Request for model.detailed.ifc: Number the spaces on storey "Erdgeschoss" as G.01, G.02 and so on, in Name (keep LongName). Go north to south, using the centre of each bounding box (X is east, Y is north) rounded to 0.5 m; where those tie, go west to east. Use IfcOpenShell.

First a look at what the model holds.

```python
import ifcopenshell
import ifcopenshell.util.element
import ifcopenshell.util.placement

model = ifcopenshell.open("model.detailed.ifc")
print(model.schema)
storey = next(s for s in model.by_type("IfcBuildingStorey") if s.Name == "Erdgeschoss")
spaces = [e for e in ifcopenshell.util.element.get_decomposition(storey) if e.is_a("IfcSpace")]
for e in sorted(spaces, key=lambda e: e.id()):
    origin = ifcopenshell.util.placement.get_local_placement(e.ObjectPlacement)[:3, 3]
    print(e.id(), e.Name, e.LongName, origin.round(2) + 0.0, sep=" | ")
```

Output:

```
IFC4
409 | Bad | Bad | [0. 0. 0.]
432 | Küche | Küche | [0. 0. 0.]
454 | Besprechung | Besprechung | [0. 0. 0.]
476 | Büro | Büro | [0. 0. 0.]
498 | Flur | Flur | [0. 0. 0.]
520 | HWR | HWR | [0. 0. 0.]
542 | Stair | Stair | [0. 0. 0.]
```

```python
import ifcopenshell
import ifcopenshell.geom
import ifcopenshell.util.element
import ifcopenshell.util.shape

model = ifcopenshell.open("model.detailed.ifc")
settings = ifcopenshell.geom.settings()
settings.set("use-world-coords", True)


def centre(element):
    shape = ifcopenshell.geom.create_shape(settings, element)
    return ifcopenshell.util.shape.get_bbox_centroid(shape.geometry)


storey = next(s for s in model.by_type("IfcBuildingStorey") if s.Name == "Erdgeschoss")
spaces = [e for e in ifcopenshell.util.element.get_decomposition(storey) if e.is_a("IfcSpace")]

# Insertion points can sit at a corner or the storey origin, so sort by the geometry (in metres).
centres = {e: centre(e) for e in spaces}
spaces.sort(key=lambda e: (-round(centres[e][1] / 0.5), centres[e][0]))

for i, e in enumerate(spaces, start=1):
    number = f"G.{i:02d}"
    e.Name = number
    print(e.id(), number)

model.write("model.detailed_rev.ifc")
```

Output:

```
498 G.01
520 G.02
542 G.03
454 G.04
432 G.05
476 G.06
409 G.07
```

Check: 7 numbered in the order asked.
